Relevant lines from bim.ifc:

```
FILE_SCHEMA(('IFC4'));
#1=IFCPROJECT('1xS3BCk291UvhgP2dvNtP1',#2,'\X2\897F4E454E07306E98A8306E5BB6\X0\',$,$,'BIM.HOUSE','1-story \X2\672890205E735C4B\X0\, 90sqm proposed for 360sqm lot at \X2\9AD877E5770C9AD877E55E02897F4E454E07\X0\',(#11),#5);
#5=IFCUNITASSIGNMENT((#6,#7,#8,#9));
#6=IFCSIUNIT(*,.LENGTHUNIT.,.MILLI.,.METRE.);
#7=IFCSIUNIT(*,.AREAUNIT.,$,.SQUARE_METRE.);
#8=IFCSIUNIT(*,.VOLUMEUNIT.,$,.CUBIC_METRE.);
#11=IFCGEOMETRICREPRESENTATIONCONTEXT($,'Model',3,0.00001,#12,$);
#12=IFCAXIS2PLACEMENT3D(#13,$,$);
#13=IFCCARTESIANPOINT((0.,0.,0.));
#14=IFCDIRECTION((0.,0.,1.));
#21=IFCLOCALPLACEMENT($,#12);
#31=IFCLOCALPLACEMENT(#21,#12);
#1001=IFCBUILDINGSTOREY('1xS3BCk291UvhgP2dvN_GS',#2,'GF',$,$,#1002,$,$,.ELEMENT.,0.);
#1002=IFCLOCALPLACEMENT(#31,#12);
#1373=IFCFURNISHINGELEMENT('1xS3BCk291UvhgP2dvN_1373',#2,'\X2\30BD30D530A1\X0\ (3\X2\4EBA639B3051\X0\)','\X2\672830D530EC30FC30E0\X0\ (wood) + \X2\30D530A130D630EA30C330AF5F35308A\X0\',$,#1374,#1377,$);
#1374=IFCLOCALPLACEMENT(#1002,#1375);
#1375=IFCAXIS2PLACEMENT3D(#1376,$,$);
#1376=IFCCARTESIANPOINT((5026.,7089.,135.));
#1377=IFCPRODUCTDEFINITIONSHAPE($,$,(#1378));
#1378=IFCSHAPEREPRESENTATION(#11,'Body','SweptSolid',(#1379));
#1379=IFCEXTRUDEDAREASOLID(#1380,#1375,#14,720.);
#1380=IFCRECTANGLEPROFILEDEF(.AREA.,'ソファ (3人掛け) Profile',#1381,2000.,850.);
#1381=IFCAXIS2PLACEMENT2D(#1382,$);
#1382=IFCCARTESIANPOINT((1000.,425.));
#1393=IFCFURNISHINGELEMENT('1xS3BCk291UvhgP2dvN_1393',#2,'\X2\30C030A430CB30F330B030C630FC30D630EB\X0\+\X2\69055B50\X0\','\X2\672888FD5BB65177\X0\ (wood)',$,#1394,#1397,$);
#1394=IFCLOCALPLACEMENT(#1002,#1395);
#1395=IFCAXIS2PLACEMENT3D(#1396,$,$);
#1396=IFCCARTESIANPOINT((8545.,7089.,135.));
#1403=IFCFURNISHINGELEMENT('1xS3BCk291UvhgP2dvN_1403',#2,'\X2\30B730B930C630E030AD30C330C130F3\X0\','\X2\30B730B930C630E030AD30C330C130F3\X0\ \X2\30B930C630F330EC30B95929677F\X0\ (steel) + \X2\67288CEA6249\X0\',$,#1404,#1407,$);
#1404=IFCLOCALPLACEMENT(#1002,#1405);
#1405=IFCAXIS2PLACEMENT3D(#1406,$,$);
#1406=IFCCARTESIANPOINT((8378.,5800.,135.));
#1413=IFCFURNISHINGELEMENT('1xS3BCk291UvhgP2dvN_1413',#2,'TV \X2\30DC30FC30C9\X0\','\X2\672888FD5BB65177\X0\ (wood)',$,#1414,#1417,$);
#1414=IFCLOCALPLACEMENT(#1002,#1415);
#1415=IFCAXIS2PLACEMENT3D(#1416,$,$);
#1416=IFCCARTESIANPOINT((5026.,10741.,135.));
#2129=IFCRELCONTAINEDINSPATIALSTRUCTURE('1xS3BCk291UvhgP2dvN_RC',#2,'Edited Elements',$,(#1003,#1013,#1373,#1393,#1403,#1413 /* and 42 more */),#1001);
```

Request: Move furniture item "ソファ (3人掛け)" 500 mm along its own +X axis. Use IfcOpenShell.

```python
import ifcopenshell
import ifcopenshell.api.geometry
import ifcopenshell.util.placement

model = ifcopenshell.open("bim.ifc")

item = model.by_id(1373)
matrix = ifcopenshell.util.placement.get_local_placement(item.ObjectPlacement)
matrix[:3, 3] += matrix[:3, 0] * 500.0
ifcopenshell.api.geometry.edit_object_placement(model, product=item, matrix=matrix, is_si=False)

print(ifcopenshell.util.placement.get_local_placement(item.ObjectPlacement).round(3) + 0.0)

model.write("bim_updated.ifc")
```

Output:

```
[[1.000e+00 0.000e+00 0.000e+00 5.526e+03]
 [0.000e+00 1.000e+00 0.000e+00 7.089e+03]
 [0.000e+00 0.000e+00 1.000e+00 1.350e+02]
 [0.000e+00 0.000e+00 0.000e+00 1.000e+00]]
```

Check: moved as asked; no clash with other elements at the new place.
